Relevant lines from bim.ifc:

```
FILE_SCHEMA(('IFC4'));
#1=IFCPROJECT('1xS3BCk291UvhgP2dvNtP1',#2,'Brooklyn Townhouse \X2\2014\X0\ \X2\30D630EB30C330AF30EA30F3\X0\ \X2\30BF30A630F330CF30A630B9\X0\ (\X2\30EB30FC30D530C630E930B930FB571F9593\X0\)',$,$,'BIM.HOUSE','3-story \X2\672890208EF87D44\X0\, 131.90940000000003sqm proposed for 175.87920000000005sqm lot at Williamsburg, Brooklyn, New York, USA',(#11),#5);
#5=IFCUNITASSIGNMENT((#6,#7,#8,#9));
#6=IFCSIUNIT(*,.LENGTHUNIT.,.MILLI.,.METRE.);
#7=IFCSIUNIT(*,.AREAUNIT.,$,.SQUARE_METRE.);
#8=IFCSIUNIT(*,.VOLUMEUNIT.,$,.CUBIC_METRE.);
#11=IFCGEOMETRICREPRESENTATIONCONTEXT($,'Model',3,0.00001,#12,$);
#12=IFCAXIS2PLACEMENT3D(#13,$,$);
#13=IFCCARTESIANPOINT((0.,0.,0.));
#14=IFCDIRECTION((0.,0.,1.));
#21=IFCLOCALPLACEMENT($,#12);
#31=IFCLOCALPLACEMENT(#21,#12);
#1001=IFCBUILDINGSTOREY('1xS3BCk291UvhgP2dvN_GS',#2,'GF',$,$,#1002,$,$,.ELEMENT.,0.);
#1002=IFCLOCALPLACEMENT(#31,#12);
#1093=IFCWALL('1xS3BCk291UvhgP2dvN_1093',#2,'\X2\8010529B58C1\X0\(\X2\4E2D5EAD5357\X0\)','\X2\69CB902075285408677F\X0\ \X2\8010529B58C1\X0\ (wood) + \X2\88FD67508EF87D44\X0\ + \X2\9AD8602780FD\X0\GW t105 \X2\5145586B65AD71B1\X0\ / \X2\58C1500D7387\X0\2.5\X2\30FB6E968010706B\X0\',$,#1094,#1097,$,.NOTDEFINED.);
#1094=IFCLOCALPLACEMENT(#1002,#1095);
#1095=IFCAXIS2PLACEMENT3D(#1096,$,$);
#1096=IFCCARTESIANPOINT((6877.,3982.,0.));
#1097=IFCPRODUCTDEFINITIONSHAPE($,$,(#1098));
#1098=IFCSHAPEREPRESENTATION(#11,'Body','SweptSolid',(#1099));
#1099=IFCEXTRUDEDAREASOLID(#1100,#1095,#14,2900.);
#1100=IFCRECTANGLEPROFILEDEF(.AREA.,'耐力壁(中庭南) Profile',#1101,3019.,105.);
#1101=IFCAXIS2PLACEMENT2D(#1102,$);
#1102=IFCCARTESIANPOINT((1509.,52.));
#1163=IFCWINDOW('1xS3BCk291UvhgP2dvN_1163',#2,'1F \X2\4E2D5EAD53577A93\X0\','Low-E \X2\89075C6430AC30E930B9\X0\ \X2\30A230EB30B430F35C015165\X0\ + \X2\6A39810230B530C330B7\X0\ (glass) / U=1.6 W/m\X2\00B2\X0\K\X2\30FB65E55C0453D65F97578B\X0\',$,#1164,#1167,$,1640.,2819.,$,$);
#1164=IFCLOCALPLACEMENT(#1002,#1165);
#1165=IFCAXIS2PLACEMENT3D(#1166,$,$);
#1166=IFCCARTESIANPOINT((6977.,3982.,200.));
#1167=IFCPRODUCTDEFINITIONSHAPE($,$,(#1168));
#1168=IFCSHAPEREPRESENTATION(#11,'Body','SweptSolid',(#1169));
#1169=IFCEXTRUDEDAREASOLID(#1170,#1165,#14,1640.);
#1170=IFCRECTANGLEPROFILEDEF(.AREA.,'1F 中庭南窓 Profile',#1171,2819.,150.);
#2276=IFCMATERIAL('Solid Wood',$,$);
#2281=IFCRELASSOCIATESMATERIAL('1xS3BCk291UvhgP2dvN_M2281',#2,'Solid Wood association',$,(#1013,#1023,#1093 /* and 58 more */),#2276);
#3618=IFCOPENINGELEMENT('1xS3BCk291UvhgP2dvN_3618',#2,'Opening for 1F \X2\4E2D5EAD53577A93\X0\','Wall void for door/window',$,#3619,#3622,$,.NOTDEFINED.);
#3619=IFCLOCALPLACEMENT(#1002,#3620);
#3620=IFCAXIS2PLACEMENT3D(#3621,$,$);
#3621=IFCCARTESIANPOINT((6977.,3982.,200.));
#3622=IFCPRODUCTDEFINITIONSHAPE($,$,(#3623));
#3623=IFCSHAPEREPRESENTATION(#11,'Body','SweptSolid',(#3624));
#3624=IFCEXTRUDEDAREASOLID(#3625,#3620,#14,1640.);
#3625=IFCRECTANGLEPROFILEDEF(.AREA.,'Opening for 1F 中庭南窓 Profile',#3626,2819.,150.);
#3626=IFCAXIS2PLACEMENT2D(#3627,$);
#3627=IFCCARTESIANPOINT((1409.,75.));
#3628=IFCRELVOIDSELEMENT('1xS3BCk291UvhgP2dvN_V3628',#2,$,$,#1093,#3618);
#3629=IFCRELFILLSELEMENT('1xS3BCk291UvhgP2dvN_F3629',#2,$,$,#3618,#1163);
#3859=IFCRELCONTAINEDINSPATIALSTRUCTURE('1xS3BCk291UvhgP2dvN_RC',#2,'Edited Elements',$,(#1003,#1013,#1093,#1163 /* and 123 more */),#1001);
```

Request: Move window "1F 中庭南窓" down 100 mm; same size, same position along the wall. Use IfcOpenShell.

```python
import numpy as np
import ifcopenshell
import ifcopenshell.api.geometry
import ifcopenshell.util.placement
import ifcopenshell.util.unit

model = ifcopenshell.open("bim.ifc")
unit_scale = ifcopenshell.util.unit.calculate_unit_scale(model)

window = model.by_guid("1xS3BCk291UvhgP2dvN_1163")
opening = window.FillsVoids[0].RelatingOpeningElement
dz = -100.0

shift = np.array([0.0, 0.0, dz])
# The window is not placed relative to its opening, so move both.
for product in (opening, window):
    matrix = ifcopenshell.util.placement.get_local_placement(product.ObjectPlacement)
    matrix[:3, 3] += shift
    ifcopenshell.api.geometry.edit_object_placement(model, product=product, matrix=matrix, is_si=False)

print(f"moved by {dz * unit_scale:+.3f} m")

model.write("bim_rev.ifc")
```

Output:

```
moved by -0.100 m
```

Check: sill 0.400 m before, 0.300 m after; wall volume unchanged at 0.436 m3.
